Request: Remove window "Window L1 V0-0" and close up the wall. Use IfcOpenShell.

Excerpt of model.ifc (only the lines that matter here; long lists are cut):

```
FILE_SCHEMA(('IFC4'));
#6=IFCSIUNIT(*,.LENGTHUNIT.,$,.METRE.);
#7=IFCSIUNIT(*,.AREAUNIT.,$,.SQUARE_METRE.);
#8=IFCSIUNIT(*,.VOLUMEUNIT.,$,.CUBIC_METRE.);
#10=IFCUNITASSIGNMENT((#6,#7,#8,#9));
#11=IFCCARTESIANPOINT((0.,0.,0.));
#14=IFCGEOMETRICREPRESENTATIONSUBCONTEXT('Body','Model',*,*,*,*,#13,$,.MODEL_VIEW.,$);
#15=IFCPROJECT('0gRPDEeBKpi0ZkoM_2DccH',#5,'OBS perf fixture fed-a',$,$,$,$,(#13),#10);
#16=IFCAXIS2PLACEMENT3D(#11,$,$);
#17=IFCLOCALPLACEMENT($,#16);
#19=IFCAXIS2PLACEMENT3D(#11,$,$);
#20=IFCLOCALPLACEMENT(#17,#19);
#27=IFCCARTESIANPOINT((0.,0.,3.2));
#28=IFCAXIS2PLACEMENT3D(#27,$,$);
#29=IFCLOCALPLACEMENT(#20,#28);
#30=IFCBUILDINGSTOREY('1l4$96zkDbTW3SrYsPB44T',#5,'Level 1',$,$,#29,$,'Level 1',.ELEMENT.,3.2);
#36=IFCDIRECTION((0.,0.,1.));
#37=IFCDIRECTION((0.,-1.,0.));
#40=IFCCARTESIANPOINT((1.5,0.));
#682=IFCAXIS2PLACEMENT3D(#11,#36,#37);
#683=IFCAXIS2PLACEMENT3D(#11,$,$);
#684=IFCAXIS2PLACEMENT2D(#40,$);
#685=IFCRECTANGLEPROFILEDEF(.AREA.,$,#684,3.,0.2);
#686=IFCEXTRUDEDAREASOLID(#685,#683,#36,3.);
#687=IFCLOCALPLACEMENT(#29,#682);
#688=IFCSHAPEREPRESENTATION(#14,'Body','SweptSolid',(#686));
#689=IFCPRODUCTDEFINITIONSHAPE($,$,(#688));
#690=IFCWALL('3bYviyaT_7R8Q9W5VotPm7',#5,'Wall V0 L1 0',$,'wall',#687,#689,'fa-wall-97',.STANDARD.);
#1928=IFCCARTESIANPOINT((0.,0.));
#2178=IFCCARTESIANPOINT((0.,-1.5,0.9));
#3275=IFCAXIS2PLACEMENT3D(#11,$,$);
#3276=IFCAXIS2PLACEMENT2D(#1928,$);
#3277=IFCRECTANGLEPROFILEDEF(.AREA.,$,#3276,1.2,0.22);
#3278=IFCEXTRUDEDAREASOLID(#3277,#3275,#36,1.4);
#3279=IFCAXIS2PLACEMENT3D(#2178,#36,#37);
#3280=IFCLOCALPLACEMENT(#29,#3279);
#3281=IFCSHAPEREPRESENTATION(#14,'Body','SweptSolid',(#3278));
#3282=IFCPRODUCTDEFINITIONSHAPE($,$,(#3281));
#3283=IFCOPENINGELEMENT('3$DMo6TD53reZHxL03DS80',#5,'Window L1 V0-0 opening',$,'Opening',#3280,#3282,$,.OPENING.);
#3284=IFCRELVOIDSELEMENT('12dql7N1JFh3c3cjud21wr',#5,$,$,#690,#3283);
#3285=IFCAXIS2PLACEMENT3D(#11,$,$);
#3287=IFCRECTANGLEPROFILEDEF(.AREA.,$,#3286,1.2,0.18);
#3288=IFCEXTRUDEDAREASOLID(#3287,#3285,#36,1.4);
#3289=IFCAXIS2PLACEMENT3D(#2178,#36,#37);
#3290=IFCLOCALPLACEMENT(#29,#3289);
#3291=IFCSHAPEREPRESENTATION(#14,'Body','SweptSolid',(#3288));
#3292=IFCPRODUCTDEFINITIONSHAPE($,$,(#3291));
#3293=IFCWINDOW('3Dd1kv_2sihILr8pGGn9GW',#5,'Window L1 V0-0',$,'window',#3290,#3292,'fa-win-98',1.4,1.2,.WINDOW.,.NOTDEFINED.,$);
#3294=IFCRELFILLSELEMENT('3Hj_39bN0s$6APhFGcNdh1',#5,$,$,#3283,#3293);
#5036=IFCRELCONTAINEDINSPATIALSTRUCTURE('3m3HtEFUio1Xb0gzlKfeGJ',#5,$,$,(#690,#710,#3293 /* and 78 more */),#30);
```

```python
import ifcopenshell
import ifcopenshell.api.feature
import ifcopenshell.api.root
import ifcopenshell.geom
import ifcopenshell.util.shape

model = ifcopenshell.open("model.ifc")
settings = ifcopenshell.geom.settings()


def volume(element):
    """Net volume in cubic metres, openings subtracted."""
    shape = ifcopenshell.geom.create_shape(settings, element)
    return ifcopenshell.util.shape.get_volume(shape.geometry)


window = model.by_id(3293)
opening = window.FillsVoids[0].RelatingOpeningElement
wall = opening.VoidsElements[0].RelatingBuildingElement
before = volume(wall)

ifcopenshell.api.root.remove_product(model, product=window)
ifcopenshell.api.feature.remove_feature(model, feature=opening)

after = volume(wall)

print(f"wall volume {before:.3f} -> {after:.3f} m3")

model.write("model-out.ifc")
```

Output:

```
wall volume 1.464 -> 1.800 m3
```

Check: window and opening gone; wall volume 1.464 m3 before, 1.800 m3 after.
